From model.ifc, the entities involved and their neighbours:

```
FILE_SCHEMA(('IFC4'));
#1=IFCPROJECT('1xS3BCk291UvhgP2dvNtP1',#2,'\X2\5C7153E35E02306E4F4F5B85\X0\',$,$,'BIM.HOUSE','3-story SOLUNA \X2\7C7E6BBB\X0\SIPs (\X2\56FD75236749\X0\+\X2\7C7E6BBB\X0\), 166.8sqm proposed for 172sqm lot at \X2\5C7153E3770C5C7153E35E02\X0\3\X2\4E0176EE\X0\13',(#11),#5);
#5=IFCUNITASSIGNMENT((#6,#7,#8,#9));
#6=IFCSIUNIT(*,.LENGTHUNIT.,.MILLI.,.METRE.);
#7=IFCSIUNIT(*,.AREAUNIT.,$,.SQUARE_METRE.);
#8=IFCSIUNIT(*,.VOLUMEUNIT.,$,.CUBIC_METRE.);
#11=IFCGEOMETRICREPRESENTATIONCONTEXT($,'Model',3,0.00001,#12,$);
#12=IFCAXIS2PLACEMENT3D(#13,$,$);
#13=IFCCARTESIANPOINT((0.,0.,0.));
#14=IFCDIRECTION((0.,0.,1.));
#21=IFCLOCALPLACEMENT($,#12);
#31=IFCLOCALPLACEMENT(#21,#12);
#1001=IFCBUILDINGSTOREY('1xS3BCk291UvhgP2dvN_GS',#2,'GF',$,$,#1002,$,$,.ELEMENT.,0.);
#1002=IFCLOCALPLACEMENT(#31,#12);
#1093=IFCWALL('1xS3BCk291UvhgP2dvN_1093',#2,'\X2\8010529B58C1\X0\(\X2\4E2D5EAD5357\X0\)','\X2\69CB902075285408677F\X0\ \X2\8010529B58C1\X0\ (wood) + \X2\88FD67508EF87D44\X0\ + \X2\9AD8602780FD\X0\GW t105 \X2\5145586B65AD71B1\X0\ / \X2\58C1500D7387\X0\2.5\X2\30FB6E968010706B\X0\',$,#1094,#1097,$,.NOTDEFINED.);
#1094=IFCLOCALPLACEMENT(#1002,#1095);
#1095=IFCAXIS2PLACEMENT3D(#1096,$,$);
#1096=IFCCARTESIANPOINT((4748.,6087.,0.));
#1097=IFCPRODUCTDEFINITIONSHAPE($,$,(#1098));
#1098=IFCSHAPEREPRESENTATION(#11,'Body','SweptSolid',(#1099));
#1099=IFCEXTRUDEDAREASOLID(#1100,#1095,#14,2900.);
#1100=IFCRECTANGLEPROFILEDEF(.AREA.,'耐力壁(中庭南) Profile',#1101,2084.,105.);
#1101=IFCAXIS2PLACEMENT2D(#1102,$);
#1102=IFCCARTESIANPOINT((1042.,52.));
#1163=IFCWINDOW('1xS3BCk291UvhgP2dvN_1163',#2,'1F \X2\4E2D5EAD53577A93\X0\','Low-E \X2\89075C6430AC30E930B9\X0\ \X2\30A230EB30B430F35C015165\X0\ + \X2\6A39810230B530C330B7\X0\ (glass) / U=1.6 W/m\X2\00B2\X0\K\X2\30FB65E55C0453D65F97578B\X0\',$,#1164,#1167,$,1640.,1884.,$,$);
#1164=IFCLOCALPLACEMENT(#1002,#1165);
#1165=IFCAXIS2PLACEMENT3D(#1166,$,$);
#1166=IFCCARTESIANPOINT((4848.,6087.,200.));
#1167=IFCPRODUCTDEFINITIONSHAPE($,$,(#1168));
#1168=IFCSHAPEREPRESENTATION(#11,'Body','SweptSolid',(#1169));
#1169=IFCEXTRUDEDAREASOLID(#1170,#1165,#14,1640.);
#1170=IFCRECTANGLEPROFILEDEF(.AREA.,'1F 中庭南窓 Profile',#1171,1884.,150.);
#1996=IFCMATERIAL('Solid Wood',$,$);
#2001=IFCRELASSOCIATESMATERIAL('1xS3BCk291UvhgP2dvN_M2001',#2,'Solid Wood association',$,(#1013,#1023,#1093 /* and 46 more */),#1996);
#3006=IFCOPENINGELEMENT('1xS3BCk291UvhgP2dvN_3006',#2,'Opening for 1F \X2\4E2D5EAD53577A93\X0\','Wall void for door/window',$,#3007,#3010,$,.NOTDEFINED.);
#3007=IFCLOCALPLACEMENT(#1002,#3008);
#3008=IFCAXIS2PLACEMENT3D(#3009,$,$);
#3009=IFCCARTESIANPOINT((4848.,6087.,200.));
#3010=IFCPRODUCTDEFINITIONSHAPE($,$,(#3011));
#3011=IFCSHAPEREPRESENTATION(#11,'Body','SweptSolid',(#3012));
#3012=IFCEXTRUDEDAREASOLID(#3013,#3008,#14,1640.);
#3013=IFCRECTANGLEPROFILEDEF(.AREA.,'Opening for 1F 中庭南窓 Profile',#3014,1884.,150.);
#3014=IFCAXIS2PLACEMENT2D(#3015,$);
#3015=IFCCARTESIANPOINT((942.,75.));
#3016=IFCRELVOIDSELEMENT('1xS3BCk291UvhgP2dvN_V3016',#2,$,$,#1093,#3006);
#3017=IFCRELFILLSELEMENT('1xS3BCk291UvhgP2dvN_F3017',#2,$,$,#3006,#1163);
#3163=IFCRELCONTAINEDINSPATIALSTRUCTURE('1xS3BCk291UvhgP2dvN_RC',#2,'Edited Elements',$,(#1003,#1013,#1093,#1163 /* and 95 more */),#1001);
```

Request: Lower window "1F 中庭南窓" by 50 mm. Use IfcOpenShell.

```python
import numpy as np
import ifcopenshell
import ifcopenshell.api.geometry
import ifcopenshell.util.placement
import ifcopenshell.util.unit

model = ifcopenshell.open("model.ifc")
unit_scale = ifcopenshell.util.unit.calculate_unit_scale(model)

window = model.by_id(1163)
opening = window.FillsVoids[0].RelatingOpeningElement
dz = -0.05 / unit_scale

shift = np.array([0.0, 0.0, dz])
# The window is not placed relative to its opening, so move both.
for product in (opening, window):
    matrix = ifcopenshell.util.placement.get_local_placement(product.ObjectPlacement)
    matrix[:3, 3] += shift
    ifcopenshell.api.geometry.edit_object_placement(model, product=product, matrix=matrix, is_si=False)

print(f"moved by {dz * unit_scale:+.3f} m")

model.write("model-out.ifc")
```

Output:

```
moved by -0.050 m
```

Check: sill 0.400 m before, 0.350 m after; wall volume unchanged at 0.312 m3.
